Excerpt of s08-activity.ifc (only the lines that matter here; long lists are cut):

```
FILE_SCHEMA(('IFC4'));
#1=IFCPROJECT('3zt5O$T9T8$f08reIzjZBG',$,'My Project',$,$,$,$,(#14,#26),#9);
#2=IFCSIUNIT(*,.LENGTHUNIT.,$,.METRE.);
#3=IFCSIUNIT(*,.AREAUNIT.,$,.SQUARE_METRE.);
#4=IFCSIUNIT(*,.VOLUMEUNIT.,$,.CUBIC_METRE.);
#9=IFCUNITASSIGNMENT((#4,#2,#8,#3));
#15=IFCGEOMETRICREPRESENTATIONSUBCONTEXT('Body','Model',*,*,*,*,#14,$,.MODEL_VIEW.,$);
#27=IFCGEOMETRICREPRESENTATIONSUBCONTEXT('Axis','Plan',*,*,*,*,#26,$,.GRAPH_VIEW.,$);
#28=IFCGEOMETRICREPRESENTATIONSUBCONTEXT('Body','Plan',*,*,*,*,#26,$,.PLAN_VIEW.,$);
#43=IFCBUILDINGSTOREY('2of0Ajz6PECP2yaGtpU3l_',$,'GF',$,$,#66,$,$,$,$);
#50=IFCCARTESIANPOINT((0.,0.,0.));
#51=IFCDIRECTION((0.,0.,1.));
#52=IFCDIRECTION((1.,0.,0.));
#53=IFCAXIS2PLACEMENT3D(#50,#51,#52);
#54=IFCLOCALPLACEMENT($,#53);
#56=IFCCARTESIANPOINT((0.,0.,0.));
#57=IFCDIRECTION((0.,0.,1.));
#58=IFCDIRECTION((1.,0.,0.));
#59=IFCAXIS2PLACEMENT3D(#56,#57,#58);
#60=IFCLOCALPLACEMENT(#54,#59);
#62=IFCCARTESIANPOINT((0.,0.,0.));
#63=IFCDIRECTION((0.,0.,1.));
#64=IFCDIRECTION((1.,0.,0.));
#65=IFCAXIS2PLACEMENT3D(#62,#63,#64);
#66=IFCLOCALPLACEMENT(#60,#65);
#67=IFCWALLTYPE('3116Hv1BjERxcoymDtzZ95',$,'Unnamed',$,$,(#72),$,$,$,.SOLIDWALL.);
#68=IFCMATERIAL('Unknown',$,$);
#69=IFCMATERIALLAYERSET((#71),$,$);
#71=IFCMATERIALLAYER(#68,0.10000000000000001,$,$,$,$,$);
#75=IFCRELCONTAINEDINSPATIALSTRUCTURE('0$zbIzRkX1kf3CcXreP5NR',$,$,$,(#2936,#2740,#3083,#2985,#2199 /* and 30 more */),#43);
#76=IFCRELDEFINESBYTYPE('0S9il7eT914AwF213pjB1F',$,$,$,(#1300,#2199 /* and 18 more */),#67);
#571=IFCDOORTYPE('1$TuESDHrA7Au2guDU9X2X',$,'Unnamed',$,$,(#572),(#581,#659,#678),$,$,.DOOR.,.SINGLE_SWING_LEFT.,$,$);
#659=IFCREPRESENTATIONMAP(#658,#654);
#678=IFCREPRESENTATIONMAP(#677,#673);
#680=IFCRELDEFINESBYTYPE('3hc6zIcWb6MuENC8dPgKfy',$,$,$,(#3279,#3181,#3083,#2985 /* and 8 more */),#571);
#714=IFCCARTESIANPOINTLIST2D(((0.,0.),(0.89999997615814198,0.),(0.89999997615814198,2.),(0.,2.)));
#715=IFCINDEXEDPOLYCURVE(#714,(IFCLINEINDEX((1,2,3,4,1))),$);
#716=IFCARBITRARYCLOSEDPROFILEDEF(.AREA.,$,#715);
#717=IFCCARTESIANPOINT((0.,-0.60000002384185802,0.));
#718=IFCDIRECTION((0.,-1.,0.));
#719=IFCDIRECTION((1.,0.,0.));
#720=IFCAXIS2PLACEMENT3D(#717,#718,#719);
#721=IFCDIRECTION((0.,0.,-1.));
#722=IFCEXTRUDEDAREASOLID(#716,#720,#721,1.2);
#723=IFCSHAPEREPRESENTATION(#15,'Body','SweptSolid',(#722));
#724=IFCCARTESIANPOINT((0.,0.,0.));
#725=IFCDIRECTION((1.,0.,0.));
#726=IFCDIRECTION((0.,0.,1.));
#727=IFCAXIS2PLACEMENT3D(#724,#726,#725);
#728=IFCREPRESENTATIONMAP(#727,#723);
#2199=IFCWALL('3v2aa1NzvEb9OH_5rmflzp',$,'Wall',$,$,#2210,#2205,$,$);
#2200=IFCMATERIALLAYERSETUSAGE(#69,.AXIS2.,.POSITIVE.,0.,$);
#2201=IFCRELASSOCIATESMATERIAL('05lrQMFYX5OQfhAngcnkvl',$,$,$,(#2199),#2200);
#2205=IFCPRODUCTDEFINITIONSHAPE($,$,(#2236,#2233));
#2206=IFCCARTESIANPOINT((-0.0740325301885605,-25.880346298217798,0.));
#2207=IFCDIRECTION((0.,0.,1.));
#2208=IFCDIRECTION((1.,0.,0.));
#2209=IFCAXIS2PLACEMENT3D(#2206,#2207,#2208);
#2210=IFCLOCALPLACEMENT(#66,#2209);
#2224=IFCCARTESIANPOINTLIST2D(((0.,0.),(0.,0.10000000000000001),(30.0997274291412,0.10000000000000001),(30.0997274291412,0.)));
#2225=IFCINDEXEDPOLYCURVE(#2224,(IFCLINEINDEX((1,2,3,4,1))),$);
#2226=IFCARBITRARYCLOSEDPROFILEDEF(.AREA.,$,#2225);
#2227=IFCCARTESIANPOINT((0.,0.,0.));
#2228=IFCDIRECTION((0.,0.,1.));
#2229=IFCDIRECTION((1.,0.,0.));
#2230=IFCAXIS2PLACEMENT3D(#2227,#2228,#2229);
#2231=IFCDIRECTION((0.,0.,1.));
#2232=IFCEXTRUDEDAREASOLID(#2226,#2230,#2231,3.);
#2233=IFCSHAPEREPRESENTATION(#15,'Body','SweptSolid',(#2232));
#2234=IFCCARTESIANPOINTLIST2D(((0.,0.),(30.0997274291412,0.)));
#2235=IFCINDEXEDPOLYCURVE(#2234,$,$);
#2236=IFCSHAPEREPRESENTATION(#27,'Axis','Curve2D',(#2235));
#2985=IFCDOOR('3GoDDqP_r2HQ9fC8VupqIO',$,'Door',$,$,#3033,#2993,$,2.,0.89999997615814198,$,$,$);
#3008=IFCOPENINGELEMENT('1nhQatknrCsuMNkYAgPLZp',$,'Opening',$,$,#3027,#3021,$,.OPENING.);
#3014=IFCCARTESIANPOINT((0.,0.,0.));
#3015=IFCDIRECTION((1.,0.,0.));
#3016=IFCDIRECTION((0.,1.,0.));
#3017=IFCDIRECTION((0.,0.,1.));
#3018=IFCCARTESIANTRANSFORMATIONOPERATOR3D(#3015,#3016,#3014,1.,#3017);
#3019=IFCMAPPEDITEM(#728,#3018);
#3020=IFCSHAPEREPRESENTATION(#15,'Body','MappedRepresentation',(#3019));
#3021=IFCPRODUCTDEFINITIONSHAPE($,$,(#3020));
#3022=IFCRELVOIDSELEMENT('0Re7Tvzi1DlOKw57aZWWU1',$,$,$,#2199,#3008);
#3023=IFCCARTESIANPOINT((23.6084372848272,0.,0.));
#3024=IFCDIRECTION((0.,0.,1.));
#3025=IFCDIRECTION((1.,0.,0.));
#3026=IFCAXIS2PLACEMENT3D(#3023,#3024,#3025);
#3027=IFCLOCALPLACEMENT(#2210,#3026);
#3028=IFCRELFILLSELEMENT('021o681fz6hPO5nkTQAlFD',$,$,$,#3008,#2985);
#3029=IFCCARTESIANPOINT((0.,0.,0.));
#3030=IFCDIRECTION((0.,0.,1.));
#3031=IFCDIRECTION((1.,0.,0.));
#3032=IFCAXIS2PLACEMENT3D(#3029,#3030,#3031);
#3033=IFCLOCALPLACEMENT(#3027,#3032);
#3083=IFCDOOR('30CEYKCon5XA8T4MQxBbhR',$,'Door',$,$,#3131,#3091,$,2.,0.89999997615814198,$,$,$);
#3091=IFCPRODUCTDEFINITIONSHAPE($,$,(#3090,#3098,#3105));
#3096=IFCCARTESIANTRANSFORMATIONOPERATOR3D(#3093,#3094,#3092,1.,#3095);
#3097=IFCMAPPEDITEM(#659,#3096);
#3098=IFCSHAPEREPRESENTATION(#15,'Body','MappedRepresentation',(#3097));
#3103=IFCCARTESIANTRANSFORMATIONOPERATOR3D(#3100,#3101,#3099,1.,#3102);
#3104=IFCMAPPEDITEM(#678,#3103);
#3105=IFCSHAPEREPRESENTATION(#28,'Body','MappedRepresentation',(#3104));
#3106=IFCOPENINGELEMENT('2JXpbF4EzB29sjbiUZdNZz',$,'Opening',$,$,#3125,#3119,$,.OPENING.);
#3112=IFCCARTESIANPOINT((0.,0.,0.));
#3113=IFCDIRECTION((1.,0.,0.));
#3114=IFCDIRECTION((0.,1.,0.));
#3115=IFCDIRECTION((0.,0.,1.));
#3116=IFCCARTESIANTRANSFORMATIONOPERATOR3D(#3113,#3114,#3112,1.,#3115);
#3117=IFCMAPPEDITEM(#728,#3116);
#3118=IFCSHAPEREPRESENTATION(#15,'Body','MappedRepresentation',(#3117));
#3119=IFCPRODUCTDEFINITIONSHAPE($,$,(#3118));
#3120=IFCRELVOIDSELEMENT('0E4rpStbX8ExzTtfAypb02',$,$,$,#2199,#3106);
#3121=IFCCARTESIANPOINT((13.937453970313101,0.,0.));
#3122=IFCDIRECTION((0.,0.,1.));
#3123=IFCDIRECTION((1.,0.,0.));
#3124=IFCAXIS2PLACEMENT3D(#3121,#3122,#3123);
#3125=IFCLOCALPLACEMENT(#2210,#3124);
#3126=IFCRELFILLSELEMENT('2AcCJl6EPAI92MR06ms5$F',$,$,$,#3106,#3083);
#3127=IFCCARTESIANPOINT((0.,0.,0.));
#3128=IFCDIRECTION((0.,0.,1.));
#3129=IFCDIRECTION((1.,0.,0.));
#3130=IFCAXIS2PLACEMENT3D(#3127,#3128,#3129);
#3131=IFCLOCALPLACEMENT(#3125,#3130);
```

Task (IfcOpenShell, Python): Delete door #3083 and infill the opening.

```python
import ifcopenshell
import ifcopenshell.api.feature
import ifcopenshell.api.root
import ifcopenshell.geom
import ifcopenshell.util.shape

model = ifcopenshell.open("s08-activity.ifc")
settings = ifcopenshell.geom.settings()


def volume(element):
    """Net volume in cubic metres, openings subtracted."""
    shape = ifcopenshell.geom.create_shape(settings, element)
    return ifcopenshell.util.shape.get_volume(shape.geometry)


door = model.by_id(3083)
opening = door.FillsVoids[0].RelatingOpeningElement
wall = opening.VoidsElements[0].RelatingBuildingElement
before = volume(wall)

ifcopenshell.api.root.remove_product(model, product=door)
ifcopenshell.api.feature.remove_feature(model, feature=opening)

after = volume(wall)

print(f"wall volume {before:.3f} -> {after:.3f} m3")

model.write("s08-activity_v2.ifc")
```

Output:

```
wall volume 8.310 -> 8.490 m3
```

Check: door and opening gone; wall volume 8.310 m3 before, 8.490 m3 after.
